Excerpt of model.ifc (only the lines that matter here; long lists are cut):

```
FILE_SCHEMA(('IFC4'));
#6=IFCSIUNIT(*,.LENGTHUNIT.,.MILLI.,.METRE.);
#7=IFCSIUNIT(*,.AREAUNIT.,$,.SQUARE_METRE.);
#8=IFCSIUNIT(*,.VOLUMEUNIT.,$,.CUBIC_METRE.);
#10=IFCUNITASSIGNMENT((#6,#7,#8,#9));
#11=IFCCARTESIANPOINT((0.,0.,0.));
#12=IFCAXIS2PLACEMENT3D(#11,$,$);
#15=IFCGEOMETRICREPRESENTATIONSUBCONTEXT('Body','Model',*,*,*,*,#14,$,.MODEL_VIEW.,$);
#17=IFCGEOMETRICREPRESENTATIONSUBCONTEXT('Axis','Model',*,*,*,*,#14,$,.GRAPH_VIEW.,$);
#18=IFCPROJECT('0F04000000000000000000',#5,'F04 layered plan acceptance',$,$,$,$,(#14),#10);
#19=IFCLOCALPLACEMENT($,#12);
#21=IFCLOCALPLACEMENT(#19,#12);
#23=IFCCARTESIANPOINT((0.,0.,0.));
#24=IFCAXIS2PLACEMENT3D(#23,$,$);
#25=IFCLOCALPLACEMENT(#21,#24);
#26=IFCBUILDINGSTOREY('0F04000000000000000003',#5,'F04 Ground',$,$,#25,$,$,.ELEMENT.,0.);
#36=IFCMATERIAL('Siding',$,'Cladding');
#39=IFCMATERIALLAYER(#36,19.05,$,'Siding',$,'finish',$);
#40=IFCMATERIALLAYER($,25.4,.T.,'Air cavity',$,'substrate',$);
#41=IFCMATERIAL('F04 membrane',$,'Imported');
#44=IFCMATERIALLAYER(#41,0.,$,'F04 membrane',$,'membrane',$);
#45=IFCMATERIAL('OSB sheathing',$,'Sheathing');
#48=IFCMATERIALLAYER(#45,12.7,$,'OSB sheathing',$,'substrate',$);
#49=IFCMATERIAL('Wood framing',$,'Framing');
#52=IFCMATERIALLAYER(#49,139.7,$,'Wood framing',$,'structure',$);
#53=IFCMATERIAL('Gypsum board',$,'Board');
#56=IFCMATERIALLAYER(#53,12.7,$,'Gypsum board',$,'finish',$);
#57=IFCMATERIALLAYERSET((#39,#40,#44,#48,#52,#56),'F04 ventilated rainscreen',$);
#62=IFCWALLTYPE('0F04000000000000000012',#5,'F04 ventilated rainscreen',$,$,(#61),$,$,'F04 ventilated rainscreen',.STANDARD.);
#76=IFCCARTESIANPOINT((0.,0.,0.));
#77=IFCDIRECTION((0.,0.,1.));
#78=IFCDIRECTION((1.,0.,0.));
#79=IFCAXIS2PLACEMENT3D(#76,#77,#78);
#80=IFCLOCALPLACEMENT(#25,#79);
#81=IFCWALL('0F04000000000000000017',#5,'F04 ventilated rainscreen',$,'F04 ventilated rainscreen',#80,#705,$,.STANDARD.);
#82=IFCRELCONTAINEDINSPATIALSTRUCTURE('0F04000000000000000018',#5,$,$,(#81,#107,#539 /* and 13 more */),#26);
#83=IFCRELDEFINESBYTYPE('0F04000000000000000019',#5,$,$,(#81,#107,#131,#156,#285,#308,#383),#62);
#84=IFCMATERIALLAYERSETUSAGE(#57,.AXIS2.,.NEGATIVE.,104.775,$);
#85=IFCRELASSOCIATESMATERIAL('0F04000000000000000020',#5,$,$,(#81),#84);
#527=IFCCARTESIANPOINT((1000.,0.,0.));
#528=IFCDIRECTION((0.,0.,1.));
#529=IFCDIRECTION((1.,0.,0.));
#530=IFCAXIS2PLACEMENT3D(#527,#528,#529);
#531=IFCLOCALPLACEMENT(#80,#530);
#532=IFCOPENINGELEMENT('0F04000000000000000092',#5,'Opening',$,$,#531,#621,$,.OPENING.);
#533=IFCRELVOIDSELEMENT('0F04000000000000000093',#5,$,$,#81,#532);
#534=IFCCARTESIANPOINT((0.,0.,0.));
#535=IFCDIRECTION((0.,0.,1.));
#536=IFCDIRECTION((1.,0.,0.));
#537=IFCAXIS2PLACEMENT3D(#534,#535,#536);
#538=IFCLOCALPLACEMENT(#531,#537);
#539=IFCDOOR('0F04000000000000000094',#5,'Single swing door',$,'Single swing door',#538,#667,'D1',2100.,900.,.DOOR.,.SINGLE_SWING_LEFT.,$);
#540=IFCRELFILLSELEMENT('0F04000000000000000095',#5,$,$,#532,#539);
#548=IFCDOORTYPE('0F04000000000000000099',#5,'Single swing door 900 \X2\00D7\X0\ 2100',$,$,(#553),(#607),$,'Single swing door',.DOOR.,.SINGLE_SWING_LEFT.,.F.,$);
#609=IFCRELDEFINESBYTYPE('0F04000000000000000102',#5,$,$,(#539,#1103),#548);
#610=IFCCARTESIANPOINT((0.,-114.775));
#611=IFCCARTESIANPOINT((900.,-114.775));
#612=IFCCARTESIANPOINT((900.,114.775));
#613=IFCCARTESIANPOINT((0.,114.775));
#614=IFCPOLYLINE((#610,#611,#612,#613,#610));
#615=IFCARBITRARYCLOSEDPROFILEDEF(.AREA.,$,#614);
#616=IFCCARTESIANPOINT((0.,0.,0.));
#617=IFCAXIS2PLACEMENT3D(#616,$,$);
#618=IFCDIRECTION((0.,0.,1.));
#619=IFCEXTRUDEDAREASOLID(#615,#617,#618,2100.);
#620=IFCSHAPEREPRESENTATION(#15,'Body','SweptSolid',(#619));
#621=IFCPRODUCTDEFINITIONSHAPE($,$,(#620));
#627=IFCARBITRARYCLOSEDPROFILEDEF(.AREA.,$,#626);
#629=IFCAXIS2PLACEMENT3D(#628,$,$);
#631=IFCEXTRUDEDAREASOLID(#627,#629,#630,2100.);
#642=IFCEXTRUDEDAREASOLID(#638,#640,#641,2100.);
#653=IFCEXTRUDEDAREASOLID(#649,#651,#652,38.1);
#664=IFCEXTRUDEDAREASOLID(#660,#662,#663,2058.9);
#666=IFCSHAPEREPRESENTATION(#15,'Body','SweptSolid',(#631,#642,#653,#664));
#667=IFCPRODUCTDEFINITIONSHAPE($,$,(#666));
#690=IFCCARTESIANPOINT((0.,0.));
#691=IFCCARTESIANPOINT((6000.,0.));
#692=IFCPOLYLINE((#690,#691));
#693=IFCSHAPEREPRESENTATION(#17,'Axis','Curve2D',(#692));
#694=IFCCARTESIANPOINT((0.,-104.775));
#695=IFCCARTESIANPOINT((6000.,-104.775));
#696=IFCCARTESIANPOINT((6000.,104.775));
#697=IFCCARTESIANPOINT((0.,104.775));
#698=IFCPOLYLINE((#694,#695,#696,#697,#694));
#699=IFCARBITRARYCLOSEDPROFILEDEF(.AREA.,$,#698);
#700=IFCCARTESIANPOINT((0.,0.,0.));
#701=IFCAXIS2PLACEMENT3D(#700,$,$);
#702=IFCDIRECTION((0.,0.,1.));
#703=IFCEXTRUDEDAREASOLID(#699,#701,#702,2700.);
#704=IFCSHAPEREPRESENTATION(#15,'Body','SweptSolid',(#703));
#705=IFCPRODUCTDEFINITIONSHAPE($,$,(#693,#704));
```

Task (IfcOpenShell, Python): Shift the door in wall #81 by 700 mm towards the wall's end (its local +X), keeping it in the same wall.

```python
import ifcopenshell
import ifcopenshell.api.geometry
import ifcopenshell.util.placement
import ifcopenshell.util.unit

model = ifcopenshell.open("model.ifc")
unit_scale = ifcopenshell.util.unit.calculate_unit_scale(model)

door = model.by_guid("0F04000000000000000094")
opening = door.FillsVoids[0].RelatingOpeningElement
wall = opening.VoidsElements[0].RelatingBuildingElement

wall_matrix = ifcopenshell.util.placement.get_local_placement(wall.ObjectPlacement)
shift = wall_matrix[:3, 0] * 0.7 / unit_scale
before = ifcopenshell.util.placement.get_local_placement(door.ObjectPlacement)[:3, 3].copy()

# The door is placed relative to its opening, so it follows when the opening moves.
matrix = ifcopenshell.util.placement.get_local_placement(opening.ObjectPlacement)
matrix[:3, 3] += shift
ifcopenshell.api.geometry.edit_object_placement(
    model, product=opening, matrix=matrix, is_si=False, should_transform_children=True
)

after = ifcopenshell.util.placement.get_local_placement(door.ObjectPlacement)[:3, 3]
print("door moved by", (after - before).round(3) + 0.0)

model.write("model_rev.ifc")
```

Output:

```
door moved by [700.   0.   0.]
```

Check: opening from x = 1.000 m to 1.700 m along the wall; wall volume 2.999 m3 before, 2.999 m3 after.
